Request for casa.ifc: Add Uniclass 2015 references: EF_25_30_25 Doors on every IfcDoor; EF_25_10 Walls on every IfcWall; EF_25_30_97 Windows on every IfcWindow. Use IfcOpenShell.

First a look at what the model holds.

```python
import ifcopenshell

model = ifcopenshell.open("casa.ifc")
print(model.schema)
print("classifications:", [c.Name for c in model.by_type("IfcClassification")])
for ifc_class in ("IfcDoor", "IfcRoof", "IfcStair", "IfcWall", "IfcWindow"):
    print(ifc_class, len(model.by_type(ifc_class)))
```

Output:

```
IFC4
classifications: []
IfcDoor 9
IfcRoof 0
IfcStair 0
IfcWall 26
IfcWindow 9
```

```python
import ifcopenshell
import ifcopenshell.api.classification

model = ifcopenshell.open("casa.ifc")

system = ifcopenshell.api.classification.add_classification(model, classification="Uniclass 2015")

codes = {
    "IfcDoor": ("EF_25_30_25", "Doors"),
    "IfcWall": ("EF_25_10", "Walls"),
    "IfcWindow": ("EF_25_30_97", "Windows"),
}
for ifc_class, (code, name) in codes.items():
    products = model.by_type(ifc_class)
    ifcopenshell.api.classification.add_reference(
        model, products=products, classification=system, identification=code, name=name
    )
    print(code, len(products))

model.write("casa_rev.ifc")
```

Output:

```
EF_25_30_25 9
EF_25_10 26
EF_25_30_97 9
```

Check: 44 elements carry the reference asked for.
